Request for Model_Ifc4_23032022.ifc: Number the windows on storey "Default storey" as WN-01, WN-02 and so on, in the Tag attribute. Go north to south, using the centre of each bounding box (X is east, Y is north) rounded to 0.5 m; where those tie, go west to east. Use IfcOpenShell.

First a look at what the model holds.

```python
import ifcopenshell
import ifcopenshell.util.element
import ifcopenshell.util.placement

model = ifcopenshell.open("Model_Ifc4_23032022.ifc")
print(model.schema)
storey = next(s for s in model.by_type("IfcBuildingStorey") if s.Name == "Default storey")
windows = [e for e in ifcopenshell.util.element.get_decomposition(storey) if e.is_a("IfcWindow")]
for e in sorted(windows, key=lambda e: e.id()):
    origin = ifcopenshell.util.placement.get_local_placement(e.ObjectPlacement)[:3, 3]
    print(e.id(), e.Tag, e.Name, origin.round(2) + 0.0, sep=" | ")
```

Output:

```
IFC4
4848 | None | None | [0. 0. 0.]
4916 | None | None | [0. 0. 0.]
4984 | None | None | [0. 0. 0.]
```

```python
import ifcopenshell
import ifcopenshell.geom
import ifcopenshell.util.element
import ifcopenshell.util.shape

model = ifcopenshell.open("Model_Ifc4_23032022.ifc")
settings = ifcopenshell.geom.settings()
settings.set("use-world-coords", True)


def centre(element):
    shape = ifcopenshell.geom.create_shape(settings, element)
    return ifcopenshell.util.shape.get_bbox_centroid(shape.geometry)


storey = next(s for s in model.by_type("IfcBuildingStorey") if s.Name == "Default storey")
windows = [e for e in ifcopenshell.util.element.get_decomposition(storey) if e.is_a("IfcWindow")]

# Insertion points can sit at a corner or the storey origin, so sort by the geometry (in metres).
centres = {e: centre(e) for e in windows}
windows.sort(key=lambda e: (-round(centres[e][1] / 0.5), centres[e][0]))

for i, e in enumerate(windows, start=1):
    number = f"WN-{i:02d}"
    e.Tag = number
    print(e.id(), number)

model.write("Model_Ifc4_23032022_v2.ifc")
```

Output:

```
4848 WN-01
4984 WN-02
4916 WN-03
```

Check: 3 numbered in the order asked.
